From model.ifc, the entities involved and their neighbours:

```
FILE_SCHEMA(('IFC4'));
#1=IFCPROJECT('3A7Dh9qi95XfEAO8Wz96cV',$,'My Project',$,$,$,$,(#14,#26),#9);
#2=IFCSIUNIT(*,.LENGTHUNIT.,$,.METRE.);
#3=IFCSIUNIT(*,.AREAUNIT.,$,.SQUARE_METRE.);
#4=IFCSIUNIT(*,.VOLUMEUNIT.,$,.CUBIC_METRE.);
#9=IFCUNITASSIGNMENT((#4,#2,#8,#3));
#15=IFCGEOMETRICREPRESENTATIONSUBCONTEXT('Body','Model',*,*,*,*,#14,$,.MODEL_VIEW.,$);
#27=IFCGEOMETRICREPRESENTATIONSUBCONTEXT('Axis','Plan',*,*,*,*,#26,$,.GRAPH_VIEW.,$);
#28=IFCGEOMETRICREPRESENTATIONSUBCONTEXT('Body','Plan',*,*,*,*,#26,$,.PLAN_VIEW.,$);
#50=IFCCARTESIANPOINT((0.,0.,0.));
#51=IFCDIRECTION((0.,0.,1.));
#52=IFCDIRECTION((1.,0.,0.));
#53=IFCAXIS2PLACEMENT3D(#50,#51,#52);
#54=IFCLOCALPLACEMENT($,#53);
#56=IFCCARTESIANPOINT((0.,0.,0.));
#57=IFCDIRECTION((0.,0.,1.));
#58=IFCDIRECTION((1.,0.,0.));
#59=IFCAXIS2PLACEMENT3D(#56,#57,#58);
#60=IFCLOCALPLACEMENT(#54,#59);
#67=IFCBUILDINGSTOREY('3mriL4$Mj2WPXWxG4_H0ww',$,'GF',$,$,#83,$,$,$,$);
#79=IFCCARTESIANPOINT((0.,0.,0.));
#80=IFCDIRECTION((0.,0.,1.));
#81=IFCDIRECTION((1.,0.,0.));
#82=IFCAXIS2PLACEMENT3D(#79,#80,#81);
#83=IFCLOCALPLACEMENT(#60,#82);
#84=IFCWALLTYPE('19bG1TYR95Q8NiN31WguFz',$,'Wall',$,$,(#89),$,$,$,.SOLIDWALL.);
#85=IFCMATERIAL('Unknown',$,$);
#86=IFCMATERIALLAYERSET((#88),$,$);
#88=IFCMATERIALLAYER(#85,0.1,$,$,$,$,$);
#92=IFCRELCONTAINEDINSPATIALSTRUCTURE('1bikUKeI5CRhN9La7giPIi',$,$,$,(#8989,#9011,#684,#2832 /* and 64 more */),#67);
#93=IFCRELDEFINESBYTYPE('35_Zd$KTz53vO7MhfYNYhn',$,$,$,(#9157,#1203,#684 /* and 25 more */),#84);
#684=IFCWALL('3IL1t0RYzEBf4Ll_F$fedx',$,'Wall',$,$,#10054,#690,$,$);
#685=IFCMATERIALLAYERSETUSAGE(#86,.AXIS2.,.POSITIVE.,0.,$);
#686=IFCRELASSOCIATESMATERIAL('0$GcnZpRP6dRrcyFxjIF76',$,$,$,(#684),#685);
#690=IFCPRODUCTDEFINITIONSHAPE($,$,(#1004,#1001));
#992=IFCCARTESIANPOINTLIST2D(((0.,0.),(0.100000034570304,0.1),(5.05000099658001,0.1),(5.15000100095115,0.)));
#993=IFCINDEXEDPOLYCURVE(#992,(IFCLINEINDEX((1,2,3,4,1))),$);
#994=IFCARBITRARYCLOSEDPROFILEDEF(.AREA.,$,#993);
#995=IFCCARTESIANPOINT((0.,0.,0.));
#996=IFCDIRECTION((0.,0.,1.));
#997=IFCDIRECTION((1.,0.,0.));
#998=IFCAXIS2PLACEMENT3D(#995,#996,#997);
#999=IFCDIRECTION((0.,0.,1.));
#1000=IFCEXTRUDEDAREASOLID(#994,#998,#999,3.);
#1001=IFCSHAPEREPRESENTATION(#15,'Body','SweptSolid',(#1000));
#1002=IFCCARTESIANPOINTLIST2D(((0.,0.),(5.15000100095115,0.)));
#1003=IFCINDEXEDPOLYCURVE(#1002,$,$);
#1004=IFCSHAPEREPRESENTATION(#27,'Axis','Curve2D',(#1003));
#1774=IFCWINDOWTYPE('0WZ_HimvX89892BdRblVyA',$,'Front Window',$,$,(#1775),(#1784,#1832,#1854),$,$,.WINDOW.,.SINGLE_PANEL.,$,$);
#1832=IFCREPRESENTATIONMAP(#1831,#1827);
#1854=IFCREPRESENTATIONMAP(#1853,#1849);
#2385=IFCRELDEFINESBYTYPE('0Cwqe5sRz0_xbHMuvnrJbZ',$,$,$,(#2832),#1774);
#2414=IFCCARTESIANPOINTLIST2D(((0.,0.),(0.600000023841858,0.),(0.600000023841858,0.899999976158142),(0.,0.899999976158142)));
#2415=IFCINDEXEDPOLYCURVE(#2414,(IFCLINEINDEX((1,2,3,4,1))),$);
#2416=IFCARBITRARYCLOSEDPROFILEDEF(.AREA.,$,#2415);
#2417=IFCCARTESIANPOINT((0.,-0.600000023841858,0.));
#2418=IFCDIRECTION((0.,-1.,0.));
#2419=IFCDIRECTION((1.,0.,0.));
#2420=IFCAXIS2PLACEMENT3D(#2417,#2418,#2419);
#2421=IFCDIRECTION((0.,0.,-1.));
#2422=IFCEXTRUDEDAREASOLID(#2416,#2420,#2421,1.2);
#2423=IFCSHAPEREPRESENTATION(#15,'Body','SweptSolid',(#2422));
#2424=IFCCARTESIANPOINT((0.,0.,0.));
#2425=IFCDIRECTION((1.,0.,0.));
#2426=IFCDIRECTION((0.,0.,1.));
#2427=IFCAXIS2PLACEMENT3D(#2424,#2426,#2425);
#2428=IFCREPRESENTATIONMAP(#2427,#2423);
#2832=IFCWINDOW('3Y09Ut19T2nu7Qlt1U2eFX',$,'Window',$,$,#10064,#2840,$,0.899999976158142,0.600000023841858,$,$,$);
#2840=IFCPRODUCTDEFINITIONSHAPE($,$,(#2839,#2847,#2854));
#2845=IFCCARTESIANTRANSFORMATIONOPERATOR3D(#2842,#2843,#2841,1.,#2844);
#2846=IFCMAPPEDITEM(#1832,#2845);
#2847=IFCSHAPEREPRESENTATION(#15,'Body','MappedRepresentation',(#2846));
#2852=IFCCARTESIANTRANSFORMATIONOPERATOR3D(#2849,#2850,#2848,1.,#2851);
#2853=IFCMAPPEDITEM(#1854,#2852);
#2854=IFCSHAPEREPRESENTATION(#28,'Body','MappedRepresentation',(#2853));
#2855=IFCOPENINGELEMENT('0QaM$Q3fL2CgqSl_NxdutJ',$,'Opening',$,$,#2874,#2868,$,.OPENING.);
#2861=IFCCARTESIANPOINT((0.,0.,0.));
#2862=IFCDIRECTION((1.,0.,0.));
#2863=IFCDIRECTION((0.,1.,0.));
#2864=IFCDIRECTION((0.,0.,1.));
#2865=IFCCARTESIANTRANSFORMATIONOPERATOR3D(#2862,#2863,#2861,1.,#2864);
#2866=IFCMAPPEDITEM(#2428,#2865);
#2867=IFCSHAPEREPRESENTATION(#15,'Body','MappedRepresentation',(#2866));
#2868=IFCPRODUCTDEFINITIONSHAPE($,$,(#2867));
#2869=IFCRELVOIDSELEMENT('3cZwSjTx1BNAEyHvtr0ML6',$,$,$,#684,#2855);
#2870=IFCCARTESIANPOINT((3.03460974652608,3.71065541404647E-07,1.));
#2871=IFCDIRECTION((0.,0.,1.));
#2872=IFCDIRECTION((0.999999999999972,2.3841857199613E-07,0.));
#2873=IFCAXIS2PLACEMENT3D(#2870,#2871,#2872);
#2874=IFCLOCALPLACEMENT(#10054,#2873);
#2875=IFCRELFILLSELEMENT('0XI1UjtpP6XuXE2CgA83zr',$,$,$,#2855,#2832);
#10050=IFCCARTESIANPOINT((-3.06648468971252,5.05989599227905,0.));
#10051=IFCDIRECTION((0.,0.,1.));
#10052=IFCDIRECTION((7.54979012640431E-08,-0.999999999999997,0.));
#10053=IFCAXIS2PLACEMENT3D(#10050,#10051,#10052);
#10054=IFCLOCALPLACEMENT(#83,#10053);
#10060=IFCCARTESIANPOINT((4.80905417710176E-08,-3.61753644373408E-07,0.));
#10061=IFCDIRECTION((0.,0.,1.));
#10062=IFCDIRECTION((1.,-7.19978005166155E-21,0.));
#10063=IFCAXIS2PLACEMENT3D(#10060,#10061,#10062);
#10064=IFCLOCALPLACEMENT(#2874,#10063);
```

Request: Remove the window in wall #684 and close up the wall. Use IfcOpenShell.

```python
import ifcopenshell
import ifcopenshell.api.feature
import ifcopenshell.api.root
import ifcopenshell.geom
import ifcopenshell.util.shape

model = ifcopenshell.open("model.ifc")
settings = ifcopenshell.geom.settings()


def volume(element):
    """Net volume in cubic metres, openings subtracted."""
    shape = ifcopenshell.geom.create_shape(settings, element)
    return ifcopenshell.util.shape.get_volume(shape.geometry)


window = model.by_guid("3Y09Ut19T2nu7Qlt1U2eFX")
opening = window.FillsVoids[0].RelatingOpeningElement
wall = opening.VoidsElements[0].RelatingBuildingElement
before = volume(wall)

ifcopenshell.api.root.remove_product(model, product=window)
ifcopenshell.api.feature.remove_feature(model, feature=opening)

after = volume(wall)

print(f"wall volume {before:.3f} -> {after:.3f} m3")

model.write("model_updated.ifc")
```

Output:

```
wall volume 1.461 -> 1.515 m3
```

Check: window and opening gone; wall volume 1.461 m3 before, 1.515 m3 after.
